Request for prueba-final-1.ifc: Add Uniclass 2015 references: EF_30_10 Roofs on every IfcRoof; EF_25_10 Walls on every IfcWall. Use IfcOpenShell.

First a look at what the model holds.

```python
import ifcopenshell

model = ifcopenshell.open("prueba-final-1.ifc")
print(model.schema)
print("classifications:", [c.Name for c in model.by_type("IfcClassification")])
for ifc_class in ("IfcDoor", "IfcRoof", "IfcStair", "IfcWall", "IfcWindow"):
    print(ifc_class, len(model.by_type(ifc_class)))
```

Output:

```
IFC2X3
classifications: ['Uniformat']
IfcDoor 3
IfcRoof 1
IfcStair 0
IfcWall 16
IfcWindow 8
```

```python
import ifcopenshell
import ifcopenshell.api.classification

model = ifcopenshell.open("prueba-final-1.ifc")

# IFC2X3 requires Source and Edition and has no link from the project to the system.
system = model.create_entity("IfcClassification", Source="NBS", Edition="2015", Name="Uniclass 2015")

codes = {
    "IfcRoof": ("EF_30_10", "Roofs"),
    "IfcWall": ("EF_25_10", "Walls"),
}
for ifc_class, (code, name) in codes.items():
    products = model.by_type(ifc_class)
    ifcopenshell.api.classification.add_reference(
        model, products=products, classification=system, identification=code, name=name
    )
    print(code, len(products))

model.write("prueba-final-1_edited.ifc")
```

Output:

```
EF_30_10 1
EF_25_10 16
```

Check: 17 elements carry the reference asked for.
